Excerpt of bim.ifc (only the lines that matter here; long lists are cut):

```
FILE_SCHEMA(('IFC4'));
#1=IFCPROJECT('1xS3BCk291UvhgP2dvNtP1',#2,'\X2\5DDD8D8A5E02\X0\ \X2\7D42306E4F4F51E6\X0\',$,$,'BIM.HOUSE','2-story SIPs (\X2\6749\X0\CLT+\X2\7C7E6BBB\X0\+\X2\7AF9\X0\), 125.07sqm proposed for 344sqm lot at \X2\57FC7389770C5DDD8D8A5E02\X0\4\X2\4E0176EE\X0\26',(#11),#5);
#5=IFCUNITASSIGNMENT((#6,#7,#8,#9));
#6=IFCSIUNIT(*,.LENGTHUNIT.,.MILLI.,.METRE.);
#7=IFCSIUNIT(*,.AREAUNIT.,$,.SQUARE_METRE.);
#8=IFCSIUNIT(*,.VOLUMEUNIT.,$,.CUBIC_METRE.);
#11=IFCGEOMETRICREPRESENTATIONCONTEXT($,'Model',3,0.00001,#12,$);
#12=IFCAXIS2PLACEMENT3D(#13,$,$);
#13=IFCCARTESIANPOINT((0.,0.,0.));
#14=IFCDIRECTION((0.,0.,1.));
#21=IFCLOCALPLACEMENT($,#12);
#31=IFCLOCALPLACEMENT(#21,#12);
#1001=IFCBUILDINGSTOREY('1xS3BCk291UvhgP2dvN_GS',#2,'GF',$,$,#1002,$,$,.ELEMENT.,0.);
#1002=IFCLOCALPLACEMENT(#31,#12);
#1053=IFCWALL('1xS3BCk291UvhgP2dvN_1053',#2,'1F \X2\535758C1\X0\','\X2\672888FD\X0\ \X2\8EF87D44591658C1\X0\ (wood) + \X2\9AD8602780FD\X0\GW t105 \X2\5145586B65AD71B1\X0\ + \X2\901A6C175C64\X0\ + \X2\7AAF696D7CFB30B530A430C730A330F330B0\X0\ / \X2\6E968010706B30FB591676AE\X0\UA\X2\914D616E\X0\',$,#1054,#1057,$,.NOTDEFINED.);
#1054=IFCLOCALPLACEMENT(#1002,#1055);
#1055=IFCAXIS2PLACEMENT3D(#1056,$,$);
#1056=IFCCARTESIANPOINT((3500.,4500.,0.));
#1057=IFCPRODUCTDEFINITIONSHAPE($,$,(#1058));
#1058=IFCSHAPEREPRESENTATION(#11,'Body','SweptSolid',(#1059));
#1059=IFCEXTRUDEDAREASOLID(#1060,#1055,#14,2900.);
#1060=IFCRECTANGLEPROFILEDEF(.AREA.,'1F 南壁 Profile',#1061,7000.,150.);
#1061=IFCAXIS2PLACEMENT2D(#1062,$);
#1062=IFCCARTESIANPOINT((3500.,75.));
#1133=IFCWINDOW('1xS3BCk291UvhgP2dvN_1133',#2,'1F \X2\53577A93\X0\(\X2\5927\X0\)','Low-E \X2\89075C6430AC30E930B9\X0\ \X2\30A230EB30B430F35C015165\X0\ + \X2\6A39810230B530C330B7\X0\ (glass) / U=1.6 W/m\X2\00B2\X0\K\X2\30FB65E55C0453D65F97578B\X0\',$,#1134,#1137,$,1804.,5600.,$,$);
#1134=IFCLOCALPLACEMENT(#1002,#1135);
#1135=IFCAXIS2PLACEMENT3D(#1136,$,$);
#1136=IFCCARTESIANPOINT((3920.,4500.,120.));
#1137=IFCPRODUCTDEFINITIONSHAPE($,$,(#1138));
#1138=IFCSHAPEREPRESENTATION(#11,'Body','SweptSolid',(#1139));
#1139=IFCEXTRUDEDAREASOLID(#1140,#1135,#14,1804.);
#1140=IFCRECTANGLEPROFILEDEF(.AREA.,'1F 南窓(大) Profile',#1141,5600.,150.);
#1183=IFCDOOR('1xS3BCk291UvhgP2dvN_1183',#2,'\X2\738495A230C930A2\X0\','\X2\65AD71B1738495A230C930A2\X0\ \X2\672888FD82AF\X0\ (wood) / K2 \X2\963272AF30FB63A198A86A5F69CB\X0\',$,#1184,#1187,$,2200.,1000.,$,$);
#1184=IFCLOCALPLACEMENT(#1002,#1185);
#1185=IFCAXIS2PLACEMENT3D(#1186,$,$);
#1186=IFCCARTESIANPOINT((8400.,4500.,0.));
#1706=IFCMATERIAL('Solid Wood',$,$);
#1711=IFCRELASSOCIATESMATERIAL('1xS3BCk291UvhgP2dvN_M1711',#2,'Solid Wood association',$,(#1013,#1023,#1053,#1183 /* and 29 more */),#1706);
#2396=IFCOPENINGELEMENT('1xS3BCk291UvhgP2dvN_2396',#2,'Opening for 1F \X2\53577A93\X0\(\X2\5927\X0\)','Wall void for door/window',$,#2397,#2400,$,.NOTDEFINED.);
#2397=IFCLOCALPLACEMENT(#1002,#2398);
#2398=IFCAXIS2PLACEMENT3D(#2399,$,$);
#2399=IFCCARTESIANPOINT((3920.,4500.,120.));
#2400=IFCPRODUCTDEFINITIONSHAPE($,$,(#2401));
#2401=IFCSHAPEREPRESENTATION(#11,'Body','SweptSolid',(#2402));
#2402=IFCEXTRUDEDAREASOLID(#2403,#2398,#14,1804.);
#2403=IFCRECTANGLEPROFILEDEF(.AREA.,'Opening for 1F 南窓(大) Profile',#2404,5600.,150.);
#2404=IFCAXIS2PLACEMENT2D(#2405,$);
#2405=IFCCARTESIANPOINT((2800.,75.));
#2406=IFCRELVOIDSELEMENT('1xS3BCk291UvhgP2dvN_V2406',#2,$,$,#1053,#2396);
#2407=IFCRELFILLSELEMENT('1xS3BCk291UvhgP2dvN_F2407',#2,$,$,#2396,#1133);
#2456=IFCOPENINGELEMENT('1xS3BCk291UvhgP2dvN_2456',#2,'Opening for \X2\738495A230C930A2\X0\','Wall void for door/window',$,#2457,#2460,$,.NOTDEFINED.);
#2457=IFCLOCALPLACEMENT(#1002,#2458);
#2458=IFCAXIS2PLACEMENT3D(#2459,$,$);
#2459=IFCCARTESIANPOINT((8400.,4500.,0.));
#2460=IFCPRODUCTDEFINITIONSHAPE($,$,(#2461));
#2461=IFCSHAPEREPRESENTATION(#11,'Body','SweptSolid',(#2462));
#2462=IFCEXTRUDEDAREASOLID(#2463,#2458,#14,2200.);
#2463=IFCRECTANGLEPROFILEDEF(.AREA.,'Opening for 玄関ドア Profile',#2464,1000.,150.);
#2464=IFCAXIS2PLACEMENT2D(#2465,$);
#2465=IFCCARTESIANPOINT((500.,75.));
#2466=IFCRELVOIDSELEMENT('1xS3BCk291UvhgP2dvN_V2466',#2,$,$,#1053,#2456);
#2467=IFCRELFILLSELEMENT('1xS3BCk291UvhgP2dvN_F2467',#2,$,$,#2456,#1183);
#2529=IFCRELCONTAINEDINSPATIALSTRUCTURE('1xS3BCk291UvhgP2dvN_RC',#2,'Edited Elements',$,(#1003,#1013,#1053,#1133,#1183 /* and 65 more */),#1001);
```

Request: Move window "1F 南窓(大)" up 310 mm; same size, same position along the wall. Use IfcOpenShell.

```python
import numpy as np
import ifcopenshell
import ifcopenshell.api.geometry
import ifcopenshell.util.placement
import ifcopenshell.util.unit

model = ifcopenshell.open("bim.ifc")
unit_scale = ifcopenshell.util.unit.calculate_unit_scale(model)

window = model.by_guid("1xS3BCk291UvhgP2dvN_1133")
opening = window.FillsVoids[0].RelatingOpeningElement
dz = 0.31 / unit_scale

shift = np.array([0.0, 0.0, dz])
# The window is not placed relative to its opening, so move both.
for product in (opening, window):
    matrix = ifcopenshell.util.placement.get_local_placement(product.ObjectPlacement)
    matrix[:3, 3] += shift
    ifcopenshell.api.geometry.edit_object_placement(model, product=product, matrix=matrix, is_si=False)

print(f"moved by {dz * unit_scale:+.3f} m")

model.write("bim_rev.ifc")
```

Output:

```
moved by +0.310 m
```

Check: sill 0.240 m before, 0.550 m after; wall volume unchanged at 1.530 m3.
